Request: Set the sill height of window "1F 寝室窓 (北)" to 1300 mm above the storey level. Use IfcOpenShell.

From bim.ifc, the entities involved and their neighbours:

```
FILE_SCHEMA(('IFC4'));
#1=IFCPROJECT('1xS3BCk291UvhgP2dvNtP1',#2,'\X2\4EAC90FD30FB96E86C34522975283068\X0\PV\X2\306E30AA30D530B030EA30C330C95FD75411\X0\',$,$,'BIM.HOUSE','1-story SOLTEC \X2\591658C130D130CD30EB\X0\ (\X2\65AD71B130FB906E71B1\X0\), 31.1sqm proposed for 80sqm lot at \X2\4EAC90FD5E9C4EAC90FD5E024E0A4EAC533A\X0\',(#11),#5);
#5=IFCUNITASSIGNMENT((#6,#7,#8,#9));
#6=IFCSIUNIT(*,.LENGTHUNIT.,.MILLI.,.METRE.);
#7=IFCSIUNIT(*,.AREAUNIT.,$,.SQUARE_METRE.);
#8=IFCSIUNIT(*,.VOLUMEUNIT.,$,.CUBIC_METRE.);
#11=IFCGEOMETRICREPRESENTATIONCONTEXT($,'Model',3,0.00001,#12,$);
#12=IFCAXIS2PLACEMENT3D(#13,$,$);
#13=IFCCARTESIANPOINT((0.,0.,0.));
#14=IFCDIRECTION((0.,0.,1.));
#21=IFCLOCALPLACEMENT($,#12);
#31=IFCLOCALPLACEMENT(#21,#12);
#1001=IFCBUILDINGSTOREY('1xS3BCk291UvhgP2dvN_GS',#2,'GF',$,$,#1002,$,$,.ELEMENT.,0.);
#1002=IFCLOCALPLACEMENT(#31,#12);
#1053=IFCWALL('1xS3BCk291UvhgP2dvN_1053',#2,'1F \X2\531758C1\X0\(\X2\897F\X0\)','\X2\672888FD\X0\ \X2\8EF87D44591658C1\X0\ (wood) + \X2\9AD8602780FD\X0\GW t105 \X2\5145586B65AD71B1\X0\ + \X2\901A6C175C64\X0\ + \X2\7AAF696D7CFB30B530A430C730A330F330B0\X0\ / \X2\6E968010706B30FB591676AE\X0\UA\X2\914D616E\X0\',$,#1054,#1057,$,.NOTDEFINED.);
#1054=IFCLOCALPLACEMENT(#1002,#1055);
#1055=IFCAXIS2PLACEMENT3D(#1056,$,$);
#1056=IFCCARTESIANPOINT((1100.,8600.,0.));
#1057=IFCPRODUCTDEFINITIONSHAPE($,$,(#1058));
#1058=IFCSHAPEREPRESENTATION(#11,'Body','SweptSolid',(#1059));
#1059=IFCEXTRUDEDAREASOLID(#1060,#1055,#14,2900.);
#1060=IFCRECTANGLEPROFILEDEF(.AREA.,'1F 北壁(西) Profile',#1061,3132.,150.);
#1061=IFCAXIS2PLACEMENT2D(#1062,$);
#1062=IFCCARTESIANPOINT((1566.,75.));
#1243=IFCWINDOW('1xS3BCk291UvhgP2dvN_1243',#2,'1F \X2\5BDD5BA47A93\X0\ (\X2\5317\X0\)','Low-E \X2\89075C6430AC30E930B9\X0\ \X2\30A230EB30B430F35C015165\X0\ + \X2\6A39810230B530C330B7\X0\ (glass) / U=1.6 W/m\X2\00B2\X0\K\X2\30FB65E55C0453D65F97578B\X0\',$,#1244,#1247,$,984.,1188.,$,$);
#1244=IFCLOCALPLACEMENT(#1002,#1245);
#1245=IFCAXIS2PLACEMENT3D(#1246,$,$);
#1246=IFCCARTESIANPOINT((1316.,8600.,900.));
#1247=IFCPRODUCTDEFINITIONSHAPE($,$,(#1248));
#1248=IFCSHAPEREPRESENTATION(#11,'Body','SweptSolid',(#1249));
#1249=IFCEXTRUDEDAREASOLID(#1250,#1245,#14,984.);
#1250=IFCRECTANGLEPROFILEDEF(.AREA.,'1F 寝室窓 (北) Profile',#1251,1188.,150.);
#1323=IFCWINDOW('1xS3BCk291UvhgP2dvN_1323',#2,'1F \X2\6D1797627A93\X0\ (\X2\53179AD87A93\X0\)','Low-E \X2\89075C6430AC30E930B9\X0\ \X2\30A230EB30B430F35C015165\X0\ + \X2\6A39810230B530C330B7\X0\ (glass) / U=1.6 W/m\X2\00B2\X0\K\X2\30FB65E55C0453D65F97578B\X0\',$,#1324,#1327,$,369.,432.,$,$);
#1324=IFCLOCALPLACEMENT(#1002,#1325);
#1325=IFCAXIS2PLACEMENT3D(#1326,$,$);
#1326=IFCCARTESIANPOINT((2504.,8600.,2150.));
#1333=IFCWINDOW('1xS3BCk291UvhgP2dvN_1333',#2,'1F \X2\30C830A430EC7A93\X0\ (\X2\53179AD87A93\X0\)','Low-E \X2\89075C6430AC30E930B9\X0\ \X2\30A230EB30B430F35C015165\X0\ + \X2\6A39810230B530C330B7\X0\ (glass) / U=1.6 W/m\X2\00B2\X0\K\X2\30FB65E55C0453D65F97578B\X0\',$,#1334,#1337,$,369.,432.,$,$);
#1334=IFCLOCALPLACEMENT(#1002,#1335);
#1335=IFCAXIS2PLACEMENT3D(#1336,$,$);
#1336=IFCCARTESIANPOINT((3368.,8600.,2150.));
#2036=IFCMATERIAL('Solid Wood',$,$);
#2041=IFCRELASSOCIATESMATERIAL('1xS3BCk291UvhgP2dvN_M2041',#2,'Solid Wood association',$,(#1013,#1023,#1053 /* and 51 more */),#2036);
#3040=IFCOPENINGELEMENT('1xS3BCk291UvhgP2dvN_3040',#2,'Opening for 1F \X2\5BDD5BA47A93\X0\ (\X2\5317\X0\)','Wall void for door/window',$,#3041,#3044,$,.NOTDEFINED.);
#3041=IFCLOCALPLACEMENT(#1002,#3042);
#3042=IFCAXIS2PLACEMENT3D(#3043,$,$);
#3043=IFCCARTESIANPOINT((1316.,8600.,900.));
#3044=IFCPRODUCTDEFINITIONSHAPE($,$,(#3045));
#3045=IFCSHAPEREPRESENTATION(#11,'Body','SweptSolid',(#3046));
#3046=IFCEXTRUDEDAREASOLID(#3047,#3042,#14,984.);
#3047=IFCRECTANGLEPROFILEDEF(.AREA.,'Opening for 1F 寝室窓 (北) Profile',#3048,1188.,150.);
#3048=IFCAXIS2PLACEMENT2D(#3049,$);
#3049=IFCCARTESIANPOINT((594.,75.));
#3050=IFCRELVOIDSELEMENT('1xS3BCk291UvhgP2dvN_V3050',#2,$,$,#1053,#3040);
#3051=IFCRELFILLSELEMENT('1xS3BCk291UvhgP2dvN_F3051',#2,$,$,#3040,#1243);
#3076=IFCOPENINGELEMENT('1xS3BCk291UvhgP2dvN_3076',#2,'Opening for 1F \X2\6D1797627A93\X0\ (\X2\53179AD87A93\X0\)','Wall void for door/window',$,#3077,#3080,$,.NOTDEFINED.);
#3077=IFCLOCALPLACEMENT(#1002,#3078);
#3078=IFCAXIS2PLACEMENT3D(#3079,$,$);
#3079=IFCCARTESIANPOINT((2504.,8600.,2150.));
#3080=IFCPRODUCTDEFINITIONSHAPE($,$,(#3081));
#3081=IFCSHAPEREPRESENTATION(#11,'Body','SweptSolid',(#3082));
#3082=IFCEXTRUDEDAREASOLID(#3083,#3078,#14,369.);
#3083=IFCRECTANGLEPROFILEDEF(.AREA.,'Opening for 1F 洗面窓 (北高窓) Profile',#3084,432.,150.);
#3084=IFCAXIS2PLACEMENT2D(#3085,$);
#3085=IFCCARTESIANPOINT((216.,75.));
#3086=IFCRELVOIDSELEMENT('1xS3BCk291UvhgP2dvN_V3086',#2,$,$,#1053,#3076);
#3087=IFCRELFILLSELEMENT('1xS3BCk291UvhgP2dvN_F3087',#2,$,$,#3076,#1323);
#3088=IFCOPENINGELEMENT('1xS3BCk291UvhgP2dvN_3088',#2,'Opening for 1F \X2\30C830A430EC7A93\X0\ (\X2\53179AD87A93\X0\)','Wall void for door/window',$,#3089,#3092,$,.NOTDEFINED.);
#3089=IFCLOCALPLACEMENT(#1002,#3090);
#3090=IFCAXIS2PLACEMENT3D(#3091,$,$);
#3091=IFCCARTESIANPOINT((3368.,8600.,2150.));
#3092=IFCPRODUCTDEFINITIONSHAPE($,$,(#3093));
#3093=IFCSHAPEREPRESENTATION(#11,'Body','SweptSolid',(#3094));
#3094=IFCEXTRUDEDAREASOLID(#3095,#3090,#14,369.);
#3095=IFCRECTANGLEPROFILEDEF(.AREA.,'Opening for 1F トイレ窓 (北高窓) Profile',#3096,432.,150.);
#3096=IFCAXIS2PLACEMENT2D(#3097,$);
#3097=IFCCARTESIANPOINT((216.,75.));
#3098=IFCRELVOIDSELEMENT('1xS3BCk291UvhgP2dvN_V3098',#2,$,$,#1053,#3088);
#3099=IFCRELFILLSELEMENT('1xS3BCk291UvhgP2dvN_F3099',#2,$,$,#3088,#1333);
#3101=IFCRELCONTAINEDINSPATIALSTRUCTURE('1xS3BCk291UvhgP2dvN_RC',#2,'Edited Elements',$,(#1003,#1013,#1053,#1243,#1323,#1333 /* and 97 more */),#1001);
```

```python
import numpy as np
import ifcopenshell
import ifcopenshell.api.geometry
import ifcopenshell.geom
import ifcopenshell.util.element
import ifcopenshell.util.placement
import ifcopenshell.util.shape
import ifcopenshell.util.unit

model = ifcopenshell.open("bim.ifc")
unit_scale = ifcopenshell.util.unit.calculate_unit_scale(model)

window = model.by_guid("1xS3BCk291UvhgP2dvN_1243")
opening = window.FillsVoids[0].RelatingOpeningElement
storey = ifcopenshell.util.element.get_container(window, ifc_class="IfcBuildingStorey")
level = ifcopenshell.util.placement.get_local_placement(storey.ObjectPlacement)[2, 3]

# The opening's origin need not be at the sill, so measure its lowest point.
shape = ifcopenshell.geom.create_shape(ifcopenshell.geom.settings(), opening)
bottom = ifcopenshell.util.shape.get_shape_bottom_elevation(shape, shape.geometry) / unit_scale
dz = level + 1300.0 - bottom

shift = np.array([0.0, 0.0, dz])
# The window is not placed relative to its opening, so move both.
for product in (opening, window):
    matrix = ifcopenshell.util.placement.get_local_placement(product.ObjectPlacement)
    matrix[:3, 3] += shift
    ifcopenshell.api.geometry.edit_object_placement(model, product=product, matrix=matrix, is_si=False)

print(f"moved by {dz * unit_scale:+.3f} m")

model.write("bim_v2.ifc")
```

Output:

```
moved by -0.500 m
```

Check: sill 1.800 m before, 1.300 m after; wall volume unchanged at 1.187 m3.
